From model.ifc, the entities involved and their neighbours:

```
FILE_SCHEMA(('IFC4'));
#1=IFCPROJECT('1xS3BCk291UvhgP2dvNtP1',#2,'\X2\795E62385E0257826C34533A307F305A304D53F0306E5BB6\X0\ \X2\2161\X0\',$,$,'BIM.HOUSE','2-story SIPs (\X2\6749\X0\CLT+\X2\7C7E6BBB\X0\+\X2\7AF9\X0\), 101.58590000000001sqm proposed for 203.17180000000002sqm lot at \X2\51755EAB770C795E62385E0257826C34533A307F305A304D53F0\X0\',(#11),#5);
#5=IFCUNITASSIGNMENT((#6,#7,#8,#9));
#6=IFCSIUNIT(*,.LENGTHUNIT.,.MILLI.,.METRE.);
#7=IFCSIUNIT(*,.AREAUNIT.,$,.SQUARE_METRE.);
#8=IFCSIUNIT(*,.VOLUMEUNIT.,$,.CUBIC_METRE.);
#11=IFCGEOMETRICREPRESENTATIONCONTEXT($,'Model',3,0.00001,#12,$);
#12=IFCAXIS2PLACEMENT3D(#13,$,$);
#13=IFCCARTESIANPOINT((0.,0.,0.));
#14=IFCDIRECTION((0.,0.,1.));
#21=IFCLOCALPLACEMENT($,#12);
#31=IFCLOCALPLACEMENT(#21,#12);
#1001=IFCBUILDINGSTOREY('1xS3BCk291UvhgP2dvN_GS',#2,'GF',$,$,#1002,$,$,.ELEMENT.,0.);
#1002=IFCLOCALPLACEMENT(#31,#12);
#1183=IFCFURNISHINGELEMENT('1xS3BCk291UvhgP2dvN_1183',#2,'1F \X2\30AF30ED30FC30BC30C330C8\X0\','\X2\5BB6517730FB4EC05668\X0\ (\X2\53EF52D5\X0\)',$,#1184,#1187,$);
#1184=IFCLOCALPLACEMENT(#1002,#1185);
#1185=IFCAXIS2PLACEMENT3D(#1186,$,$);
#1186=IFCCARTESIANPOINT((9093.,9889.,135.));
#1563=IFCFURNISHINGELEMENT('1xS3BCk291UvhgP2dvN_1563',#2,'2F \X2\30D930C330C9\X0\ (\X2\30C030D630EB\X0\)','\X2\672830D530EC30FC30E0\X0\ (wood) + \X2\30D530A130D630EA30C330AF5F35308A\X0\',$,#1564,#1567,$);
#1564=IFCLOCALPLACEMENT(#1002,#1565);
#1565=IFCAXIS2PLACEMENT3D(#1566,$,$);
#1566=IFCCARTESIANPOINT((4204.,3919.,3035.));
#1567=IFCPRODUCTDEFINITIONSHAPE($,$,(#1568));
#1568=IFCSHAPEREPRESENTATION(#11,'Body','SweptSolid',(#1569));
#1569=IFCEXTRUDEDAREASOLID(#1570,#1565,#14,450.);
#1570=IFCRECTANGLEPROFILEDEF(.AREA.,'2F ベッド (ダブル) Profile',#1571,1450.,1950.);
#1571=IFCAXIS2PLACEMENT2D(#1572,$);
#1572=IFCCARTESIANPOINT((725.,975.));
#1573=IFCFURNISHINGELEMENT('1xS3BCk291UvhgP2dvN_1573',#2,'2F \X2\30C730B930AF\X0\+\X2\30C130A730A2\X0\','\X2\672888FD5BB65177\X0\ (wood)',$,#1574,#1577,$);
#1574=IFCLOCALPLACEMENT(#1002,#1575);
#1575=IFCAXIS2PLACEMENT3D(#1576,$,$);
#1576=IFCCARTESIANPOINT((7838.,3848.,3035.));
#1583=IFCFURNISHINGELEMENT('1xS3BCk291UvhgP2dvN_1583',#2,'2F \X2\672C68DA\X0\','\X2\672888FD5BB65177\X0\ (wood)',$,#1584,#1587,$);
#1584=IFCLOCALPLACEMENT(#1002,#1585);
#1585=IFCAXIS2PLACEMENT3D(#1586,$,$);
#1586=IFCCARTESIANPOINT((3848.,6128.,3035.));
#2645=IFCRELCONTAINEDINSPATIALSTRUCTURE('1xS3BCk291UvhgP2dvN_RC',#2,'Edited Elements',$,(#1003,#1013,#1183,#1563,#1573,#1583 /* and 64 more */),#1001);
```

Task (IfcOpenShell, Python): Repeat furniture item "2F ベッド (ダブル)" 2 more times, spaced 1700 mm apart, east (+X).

```python
import numpy as np
import ifcopenshell
import ifcopenshell.api.geometry
import ifcopenshell.api.root
import ifcopenshell.util.element
import ifcopenshell.util.placement

model = ifcopenshell.open("model.ifc")


def reuse_history(source, copy):
    """copy_class also copies each property set's owner history, people and application; keep the originals."""
    for rel in copy.IsDefinedBy:
        if rel.is_a("IfcRelDefinesByProperties") and (history := rel.RelatingPropertyDefinition.OwnerHistory):
            rel.RelatingPropertyDefinition.OwnerHistory = source.OwnerHistory
            ifcopenshell.util.element.remove_deep2(model, history)


source = model.by_guid("1xS3BCk291UvhgP2dvN_1563")
base = ifcopenshell.util.placement.get_local_placement(source.ObjectPlacement)
step = np.array([1.0, 0.0, 0.0]) * 1700.0

for i in range(1, 3):
    copy = ifcopenshell.api.root.copy_class(model, product=source)
    copy.Representation = ifcopenshell.util.element.copy_deep(
        model, source.Representation, exclude=["IfcGeometricRepresentationContext", "IfcRepresentationMap"]
    )
    reuse_history(source, copy)
    matrix = base.copy()
    matrix[:3, 3] += i * step
    print("added at", matrix[:3, 3].round(3) + 0.0)
    ifcopenshell.api.geometry.edit_object_placement(model, product=copy, matrix=matrix, is_si=False)

model.write("model_updated.ifc")
```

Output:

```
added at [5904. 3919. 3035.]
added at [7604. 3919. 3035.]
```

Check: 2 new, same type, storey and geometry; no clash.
